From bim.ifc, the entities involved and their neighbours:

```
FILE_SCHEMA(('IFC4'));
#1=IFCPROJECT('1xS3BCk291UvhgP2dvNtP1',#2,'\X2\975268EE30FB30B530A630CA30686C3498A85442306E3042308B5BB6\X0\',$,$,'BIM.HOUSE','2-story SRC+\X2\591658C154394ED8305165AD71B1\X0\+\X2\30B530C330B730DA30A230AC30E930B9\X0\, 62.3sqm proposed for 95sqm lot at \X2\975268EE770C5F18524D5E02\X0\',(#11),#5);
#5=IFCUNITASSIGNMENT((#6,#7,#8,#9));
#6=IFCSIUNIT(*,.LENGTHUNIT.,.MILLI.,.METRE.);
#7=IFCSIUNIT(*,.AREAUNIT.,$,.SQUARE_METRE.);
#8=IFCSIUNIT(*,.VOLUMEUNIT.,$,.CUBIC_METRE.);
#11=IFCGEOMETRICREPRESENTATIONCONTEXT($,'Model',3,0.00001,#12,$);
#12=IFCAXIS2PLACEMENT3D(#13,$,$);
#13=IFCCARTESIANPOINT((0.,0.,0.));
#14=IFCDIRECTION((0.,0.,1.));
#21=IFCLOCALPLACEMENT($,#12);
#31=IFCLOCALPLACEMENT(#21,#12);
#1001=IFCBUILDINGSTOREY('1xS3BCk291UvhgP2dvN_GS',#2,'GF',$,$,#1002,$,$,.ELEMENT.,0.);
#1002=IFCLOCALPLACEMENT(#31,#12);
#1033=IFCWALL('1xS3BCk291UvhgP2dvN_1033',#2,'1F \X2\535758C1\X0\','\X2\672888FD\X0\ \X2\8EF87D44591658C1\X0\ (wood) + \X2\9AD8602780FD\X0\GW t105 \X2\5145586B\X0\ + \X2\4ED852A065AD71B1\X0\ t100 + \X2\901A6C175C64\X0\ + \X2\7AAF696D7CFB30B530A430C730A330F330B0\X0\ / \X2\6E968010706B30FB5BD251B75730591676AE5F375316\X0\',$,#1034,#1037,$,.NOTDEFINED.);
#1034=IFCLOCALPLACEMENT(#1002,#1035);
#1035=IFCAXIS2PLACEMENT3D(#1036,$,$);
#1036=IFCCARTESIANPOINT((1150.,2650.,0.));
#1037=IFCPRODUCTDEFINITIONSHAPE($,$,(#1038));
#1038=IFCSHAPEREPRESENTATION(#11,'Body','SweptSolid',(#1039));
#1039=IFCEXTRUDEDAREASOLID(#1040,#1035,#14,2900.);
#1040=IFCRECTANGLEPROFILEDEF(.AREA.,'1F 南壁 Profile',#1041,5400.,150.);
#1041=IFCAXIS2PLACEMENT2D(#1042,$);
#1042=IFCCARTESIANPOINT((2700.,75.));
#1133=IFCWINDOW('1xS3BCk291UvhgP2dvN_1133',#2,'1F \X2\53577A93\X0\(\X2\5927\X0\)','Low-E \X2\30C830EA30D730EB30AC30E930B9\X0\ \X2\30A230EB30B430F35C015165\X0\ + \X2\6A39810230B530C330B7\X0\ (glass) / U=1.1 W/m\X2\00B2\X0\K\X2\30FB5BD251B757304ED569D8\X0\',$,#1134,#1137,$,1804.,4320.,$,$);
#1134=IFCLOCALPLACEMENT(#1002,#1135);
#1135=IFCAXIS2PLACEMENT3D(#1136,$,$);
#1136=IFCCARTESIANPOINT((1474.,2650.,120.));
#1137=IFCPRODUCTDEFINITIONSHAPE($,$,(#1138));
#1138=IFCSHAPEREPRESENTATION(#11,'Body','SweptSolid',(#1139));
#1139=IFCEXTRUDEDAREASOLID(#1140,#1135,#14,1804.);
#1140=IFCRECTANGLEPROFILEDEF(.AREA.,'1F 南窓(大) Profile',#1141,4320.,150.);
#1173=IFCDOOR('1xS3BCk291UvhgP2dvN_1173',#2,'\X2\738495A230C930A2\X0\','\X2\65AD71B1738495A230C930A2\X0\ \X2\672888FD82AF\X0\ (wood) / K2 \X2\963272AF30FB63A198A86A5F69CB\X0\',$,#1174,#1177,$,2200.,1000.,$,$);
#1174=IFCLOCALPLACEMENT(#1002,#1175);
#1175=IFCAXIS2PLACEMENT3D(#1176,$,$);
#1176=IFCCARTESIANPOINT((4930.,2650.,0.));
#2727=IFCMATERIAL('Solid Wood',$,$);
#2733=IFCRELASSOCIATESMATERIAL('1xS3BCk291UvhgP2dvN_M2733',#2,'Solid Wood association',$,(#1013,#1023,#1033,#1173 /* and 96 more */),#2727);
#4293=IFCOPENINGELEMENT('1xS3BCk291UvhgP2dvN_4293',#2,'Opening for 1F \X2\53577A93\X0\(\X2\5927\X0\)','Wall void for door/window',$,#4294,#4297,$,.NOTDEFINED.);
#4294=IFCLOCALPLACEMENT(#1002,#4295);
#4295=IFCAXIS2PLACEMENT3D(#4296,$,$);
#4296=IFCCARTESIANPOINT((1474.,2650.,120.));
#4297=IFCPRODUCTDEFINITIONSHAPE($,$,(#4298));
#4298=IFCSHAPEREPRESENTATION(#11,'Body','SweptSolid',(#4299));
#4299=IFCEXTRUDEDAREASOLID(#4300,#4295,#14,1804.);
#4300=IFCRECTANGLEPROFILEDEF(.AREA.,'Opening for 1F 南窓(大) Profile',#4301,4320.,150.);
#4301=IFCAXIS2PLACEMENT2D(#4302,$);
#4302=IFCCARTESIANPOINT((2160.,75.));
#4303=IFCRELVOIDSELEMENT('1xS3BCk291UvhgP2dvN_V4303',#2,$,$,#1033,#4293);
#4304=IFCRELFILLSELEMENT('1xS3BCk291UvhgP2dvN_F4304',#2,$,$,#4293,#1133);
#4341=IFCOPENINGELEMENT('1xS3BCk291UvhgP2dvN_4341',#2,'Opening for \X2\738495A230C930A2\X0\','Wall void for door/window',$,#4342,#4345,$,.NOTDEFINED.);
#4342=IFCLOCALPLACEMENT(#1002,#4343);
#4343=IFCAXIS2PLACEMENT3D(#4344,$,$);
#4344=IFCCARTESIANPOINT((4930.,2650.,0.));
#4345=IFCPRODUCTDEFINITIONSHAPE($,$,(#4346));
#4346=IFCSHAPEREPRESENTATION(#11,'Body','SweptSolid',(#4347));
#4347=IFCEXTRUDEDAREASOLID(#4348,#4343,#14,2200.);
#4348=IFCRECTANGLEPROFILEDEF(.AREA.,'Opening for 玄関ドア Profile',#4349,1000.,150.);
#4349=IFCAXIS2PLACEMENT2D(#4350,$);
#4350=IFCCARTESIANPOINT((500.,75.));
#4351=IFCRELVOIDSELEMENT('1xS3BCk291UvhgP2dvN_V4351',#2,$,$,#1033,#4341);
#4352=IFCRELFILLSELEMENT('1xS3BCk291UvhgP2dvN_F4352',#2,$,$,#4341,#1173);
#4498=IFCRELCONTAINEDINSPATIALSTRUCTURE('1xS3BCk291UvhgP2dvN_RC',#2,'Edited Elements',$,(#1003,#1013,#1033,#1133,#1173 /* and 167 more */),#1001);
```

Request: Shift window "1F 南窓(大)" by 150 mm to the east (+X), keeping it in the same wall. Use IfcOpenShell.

```python
import ifcopenshell
import ifcopenshell.api.geometry
import ifcopenshell.util.placement
import ifcopenshell.util.unit

model = ifcopenshell.open("bim.ifc")
unit_scale = ifcopenshell.util.unit.calculate_unit_scale(model)

window = model.by_guid("1xS3BCk291UvhgP2dvN_1133")
opening = window.FillsVoids[0].RelatingOpeningElement
wall = opening.VoidsElements[0].RelatingBuildingElement

wall_matrix = ifcopenshell.util.placement.get_local_placement(wall.ObjectPlacement)
shift = wall_matrix[:3, 0] * 0.15 / unit_scale
before = ifcopenshell.util.placement.get_local_placement(window.ObjectPlacement)[:3, 3].copy()

# The window is not placed relative to its opening, so move both.
for product in (opening, window):
    matrix = ifcopenshell.util.placement.get_local_placement(product.ObjectPlacement)
    matrix[:3, 3] += shift
    ifcopenshell.api.geometry.edit_object_placement(model, product=product, matrix=matrix, is_si=False)

after = ifcopenshell.util.placement.get_local_placement(window.ObjectPlacement)[:3, 3]
print("window moved by", (after - before).round(3) + 0.0)

model.write("bim-out.ifc")
```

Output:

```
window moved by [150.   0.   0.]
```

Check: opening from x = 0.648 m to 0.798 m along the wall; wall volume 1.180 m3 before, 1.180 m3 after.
